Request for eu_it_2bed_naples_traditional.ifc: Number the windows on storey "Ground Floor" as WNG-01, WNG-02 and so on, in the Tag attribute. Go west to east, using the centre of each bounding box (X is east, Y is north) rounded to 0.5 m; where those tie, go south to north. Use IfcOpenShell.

First a look at what the model holds.

```python
import ifcopenshell
import ifcopenshell.util.element
import ifcopenshell.util.placement

model = ifcopenshell.open("eu_it_2bed_naples_traditional.ifc")
print(model.schema)
storey = next(s for s in model.by_type("IfcBuildingStorey") if s.Name == "Ground Floor")
windows = [e for e in ifcopenshell.util.element.get_decomposition(storey) if e.is_a("IfcWindow")]
for e in sorted(windows, key=lambda e: e.id()):
    origin = ifcopenshell.util.placement.get_local_placement(e.ObjectPlacement)[:3, 3]
    print(e.id(), e.Tag, e.Name, origin.round(2) + 0.0, sep=" | ")
```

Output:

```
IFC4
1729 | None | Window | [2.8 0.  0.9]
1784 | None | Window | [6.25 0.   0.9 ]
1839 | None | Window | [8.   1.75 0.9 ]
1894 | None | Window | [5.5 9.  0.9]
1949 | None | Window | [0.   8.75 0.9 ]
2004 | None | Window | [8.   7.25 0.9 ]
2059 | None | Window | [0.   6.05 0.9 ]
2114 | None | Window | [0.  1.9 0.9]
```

```python
import ifcopenshell
import ifcopenshell.geom
import ifcopenshell.util.element
import ifcopenshell.util.shape

model = ifcopenshell.open("eu_it_2bed_naples_traditional.ifc")
settings = ifcopenshell.geom.settings()
settings.set("use-world-coords", True)


def centre(element):
    shape = ifcopenshell.geom.create_shape(settings, element)
    return ifcopenshell.util.shape.get_bbox_centroid(shape.geometry)


storey = next(s for s in model.by_type("IfcBuildingStorey") if s.Name == "Ground Floor")
windows = [e for e in ifcopenshell.util.element.get_decomposition(storey) if e.is_a("IfcWindow")]

# Insertion points can sit at a corner or the storey origin, so sort by the geometry (in metres).
centres = {e: centre(e) for e in windows}
windows.sort(key=lambda e: (round(centres[e][0] / 0.5), centres[e][1]))

for i, e in enumerate(windows, start=1):
    number = f"WNG-{i:02d}"
    e.Tag = number
    print(e.id(), number)

model.write("eu_it_2bed_naples_traditional_updated.ifc")
```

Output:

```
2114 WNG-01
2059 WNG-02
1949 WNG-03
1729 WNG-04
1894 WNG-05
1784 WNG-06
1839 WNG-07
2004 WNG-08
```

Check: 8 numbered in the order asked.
